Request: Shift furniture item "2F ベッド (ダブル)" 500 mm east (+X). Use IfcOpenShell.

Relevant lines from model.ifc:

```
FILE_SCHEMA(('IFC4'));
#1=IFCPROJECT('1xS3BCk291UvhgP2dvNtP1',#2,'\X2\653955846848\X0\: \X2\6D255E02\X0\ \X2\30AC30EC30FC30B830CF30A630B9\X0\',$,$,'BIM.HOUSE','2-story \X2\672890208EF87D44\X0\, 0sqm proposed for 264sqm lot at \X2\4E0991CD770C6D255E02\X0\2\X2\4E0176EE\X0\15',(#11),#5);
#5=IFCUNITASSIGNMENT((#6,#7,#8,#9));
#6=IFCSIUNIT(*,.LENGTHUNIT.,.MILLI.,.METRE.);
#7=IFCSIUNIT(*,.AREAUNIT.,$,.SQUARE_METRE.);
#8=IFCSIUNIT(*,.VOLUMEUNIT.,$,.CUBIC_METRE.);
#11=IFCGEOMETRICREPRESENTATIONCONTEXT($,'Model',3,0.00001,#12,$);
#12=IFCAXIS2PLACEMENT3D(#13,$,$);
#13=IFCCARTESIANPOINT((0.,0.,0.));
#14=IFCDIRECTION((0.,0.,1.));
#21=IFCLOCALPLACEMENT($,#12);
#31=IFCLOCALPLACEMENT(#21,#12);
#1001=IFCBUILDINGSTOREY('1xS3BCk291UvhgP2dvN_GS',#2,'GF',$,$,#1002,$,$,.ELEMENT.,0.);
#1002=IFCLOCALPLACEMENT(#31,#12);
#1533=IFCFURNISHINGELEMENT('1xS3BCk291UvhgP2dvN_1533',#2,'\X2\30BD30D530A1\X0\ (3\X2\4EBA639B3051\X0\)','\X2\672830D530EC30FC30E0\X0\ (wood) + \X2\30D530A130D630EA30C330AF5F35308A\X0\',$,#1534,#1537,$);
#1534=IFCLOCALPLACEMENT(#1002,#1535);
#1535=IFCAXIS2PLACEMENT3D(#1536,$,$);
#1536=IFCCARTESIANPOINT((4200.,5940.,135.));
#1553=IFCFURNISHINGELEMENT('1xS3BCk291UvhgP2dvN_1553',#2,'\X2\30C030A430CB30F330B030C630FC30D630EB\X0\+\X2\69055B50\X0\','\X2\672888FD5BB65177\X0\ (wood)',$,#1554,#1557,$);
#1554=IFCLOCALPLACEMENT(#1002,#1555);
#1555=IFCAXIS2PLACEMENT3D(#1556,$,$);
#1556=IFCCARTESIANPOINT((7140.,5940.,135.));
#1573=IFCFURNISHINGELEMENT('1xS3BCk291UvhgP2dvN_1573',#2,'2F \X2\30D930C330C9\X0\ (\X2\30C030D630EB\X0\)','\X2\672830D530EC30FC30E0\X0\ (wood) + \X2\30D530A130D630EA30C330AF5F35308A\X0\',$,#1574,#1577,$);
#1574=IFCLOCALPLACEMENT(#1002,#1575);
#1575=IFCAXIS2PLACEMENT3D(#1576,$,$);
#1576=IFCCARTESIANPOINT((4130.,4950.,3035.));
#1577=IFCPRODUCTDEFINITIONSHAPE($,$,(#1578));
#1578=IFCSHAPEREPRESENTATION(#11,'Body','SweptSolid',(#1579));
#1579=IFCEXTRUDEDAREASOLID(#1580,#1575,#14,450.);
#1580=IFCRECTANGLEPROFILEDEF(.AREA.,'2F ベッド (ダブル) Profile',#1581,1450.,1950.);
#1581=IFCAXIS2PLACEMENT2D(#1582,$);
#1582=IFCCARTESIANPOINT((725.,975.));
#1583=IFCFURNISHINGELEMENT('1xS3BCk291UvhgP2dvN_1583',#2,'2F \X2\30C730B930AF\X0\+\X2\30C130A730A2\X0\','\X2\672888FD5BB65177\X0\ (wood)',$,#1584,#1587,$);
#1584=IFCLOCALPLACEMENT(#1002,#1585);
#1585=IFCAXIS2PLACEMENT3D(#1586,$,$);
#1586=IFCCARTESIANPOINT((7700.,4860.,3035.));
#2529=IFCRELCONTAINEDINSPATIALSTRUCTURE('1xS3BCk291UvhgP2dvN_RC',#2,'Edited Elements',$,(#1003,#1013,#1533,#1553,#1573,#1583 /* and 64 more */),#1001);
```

```python
import ifcopenshell
import ifcopenshell.api.geometry
import ifcopenshell.util.placement

model = ifcopenshell.open("model.ifc")

item = model.by_id(1573)
matrix = ifcopenshell.util.placement.get_local_placement(item.ObjectPlacement)
matrix[0, 3] += 500.0
ifcopenshell.api.geometry.edit_object_placement(model, product=item, matrix=matrix, is_si=False)

print(ifcopenshell.util.placement.get_local_placement(item.ObjectPlacement).round(3) + 0.0)

model.write("model-out.ifc")
```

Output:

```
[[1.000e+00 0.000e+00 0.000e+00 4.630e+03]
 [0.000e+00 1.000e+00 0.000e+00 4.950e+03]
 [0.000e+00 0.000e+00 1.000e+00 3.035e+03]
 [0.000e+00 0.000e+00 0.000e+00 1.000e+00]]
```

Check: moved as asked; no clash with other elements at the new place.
